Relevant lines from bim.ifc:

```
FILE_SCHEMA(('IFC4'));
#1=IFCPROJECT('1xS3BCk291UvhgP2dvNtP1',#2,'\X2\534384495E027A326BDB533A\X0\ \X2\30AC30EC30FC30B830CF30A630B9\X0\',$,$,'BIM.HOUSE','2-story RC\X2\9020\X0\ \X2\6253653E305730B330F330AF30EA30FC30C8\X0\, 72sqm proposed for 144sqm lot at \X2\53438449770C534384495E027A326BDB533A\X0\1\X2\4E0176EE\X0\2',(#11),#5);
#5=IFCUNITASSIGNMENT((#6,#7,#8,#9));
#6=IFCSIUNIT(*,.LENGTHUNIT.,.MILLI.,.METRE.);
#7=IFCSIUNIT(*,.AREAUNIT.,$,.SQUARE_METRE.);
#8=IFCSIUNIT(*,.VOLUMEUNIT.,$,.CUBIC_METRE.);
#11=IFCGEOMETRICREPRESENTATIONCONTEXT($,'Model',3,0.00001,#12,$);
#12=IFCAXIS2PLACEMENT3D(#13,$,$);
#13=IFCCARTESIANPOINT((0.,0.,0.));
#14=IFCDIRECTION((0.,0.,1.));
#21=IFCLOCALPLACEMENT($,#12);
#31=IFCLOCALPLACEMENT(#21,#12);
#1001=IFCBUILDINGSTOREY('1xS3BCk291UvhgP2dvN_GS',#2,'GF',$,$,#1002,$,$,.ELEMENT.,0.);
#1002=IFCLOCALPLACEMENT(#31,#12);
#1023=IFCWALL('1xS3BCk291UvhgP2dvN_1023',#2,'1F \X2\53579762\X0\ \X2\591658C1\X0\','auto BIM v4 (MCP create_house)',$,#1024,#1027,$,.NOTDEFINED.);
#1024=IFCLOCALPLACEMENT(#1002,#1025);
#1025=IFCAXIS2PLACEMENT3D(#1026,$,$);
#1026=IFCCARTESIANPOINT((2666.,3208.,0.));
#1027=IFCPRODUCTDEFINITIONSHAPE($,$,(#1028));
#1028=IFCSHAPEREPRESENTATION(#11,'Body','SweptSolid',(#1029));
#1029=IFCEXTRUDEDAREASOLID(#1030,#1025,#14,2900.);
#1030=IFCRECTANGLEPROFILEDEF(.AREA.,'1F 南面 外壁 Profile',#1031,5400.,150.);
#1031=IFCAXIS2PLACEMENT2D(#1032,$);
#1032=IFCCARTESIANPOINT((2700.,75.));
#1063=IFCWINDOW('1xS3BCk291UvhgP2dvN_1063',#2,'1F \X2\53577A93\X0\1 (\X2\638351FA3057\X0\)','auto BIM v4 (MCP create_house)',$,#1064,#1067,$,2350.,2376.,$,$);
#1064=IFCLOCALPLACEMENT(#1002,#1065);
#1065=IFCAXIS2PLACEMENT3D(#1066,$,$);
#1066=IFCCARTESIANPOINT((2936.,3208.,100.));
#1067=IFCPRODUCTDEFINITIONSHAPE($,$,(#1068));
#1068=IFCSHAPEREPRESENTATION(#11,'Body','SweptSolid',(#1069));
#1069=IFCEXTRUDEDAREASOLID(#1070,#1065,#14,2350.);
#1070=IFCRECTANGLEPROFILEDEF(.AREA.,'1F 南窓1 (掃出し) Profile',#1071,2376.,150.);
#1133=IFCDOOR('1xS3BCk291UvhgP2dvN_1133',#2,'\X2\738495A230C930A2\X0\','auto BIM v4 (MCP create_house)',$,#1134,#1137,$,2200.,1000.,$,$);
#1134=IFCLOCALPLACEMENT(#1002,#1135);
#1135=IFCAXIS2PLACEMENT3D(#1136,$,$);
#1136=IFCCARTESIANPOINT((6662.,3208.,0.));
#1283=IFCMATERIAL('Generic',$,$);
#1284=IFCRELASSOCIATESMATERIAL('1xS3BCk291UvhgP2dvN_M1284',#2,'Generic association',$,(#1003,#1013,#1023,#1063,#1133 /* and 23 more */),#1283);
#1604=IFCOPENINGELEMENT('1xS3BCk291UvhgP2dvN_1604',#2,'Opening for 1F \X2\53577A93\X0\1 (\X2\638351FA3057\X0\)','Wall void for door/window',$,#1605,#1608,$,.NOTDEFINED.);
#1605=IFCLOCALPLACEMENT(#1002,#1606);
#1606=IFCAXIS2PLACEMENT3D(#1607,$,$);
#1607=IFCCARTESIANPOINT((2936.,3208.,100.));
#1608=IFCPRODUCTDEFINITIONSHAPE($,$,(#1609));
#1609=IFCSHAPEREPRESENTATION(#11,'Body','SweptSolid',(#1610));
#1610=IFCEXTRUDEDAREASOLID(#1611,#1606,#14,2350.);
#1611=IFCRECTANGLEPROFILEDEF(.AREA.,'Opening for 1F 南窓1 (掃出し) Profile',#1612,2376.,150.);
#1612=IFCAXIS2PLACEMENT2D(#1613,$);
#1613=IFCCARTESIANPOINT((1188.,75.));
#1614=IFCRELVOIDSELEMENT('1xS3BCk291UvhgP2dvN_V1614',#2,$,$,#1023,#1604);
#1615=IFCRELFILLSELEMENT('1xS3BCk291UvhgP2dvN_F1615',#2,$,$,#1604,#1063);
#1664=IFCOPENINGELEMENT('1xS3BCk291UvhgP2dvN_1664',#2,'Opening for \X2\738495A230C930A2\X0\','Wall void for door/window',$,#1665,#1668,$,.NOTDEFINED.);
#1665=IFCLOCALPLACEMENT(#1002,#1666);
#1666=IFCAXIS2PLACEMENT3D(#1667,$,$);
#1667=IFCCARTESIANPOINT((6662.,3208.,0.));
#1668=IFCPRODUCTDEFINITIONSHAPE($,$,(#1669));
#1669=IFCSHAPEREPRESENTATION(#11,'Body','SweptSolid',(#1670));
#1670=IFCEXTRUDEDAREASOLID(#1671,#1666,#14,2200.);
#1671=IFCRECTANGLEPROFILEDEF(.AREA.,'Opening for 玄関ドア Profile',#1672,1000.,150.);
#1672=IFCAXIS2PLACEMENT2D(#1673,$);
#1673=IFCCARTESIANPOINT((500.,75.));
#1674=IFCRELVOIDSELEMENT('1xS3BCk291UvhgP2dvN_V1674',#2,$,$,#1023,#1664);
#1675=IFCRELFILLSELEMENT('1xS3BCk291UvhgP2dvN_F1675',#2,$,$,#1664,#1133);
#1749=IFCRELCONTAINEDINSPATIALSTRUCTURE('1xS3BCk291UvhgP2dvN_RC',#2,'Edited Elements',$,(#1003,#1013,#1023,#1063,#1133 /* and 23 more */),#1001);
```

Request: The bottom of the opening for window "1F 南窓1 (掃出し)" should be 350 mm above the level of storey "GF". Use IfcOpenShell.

```python
import numpy as np
import ifcopenshell
import ifcopenshell.api.geometry
import ifcopenshell.geom
import ifcopenshell.util.element
import ifcopenshell.util.placement
import ifcopenshell.util.shape
import ifcopenshell.util.unit

model = ifcopenshell.open("bim.ifc")
unit_scale = ifcopenshell.util.unit.calculate_unit_scale(model)

window = model.by_guid("1xS3BCk291UvhgP2dvN_1063")
opening = window.FillsVoids[0].RelatingOpeningElement
storey = ifcopenshell.util.element.get_container(window, ifc_class="IfcBuildingStorey")
level = ifcopenshell.util.placement.get_local_placement(storey.ObjectPlacement)[2, 3]

# The opening's origin need not be at the sill, so measure its lowest point.
shape = ifcopenshell.geom.create_shape(ifcopenshell.geom.settings(), opening)
bottom = ifcopenshell.util.shape.get_shape_bottom_elevation(shape, shape.geometry) / unit_scale
dz = level + 350.0 - bottom

shift = np.array([0.0, 0.0, dz])
# The window is not placed relative to its opening, so move both.
for product in (opening, window):
    matrix = ifcopenshell.util.placement.get_local_placement(product.ObjectPlacement)
    matrix[:3, 3] += shift
    ifcopenshell.api.geometry.edit_object_placement(model, product=product, matrix=matrix, is_si=False)

print(f"moved by {dz * unit_scale:+.3f} m")

model.write("bim_rev.ifc")
```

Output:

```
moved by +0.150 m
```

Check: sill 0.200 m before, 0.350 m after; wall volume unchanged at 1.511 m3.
